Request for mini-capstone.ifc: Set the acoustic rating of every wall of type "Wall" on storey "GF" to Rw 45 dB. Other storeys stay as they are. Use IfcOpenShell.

First a look at what the model holds.

```python
import ifcopenshell
import ifcopenshell.util.element

model = ifcopenshell.open("mini-capstone.ifc")
print(model.schema)
storey = next(s for s in model.by_type("IfcBuildingStorey") if s.Name == "GF")
walls = [e for e in ifcopenshell.util.element.get_decomposition(storey) if e.is_a("IfcWall")]
seen = {}
for e in walls:
    element_type = ifcopenshell.util.element.get_type(e)
    key = (element_type.Name if element_type != e and element_type else None, ifcopenshell.util.element.get_pset(e, "Pset_WallCommon", "AcousticRating"))
    seen[key] = seen.get(key, 0) + 1
for (name, value), count in sorted(seen.items(), key=str):
    print(count, "x", name, "|", value)
```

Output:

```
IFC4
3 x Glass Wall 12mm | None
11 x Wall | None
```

```python
import ifcopenshell
import ifcopenshell.api.pset
import ifcopenshell.util.element

model = ifcopenshell.open("mini-capstone.ifc")

storey = next(s for s in model.by_type("IfcBuildingStorey") if s.Name == "GF")
walls = [e for e in ifcopenshell.util.element.get_decomposition(storey) if e.is_a("IfcWall")]

count = 0
for e in walls:
    element_type = ifcopenshell.util.element.get_type(e)
    if element_type in (None, e) or element_type.Name != "Wall":
        continue
    # add_pset returns the element's existing set when there is one.
    pset = ifcopenshell.api.pset.add_pset(model, product=e, name="Pset_WallCommon")
    ifcopenshell.api.pset.edit_pset(model, pset=pset, properties={"AcousticRating": "Rw 45 dB"})
    count += 1

print(count, "walls updated")

model.write("mini-capstone_updated.ifc")
```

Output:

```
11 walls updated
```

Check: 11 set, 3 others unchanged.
